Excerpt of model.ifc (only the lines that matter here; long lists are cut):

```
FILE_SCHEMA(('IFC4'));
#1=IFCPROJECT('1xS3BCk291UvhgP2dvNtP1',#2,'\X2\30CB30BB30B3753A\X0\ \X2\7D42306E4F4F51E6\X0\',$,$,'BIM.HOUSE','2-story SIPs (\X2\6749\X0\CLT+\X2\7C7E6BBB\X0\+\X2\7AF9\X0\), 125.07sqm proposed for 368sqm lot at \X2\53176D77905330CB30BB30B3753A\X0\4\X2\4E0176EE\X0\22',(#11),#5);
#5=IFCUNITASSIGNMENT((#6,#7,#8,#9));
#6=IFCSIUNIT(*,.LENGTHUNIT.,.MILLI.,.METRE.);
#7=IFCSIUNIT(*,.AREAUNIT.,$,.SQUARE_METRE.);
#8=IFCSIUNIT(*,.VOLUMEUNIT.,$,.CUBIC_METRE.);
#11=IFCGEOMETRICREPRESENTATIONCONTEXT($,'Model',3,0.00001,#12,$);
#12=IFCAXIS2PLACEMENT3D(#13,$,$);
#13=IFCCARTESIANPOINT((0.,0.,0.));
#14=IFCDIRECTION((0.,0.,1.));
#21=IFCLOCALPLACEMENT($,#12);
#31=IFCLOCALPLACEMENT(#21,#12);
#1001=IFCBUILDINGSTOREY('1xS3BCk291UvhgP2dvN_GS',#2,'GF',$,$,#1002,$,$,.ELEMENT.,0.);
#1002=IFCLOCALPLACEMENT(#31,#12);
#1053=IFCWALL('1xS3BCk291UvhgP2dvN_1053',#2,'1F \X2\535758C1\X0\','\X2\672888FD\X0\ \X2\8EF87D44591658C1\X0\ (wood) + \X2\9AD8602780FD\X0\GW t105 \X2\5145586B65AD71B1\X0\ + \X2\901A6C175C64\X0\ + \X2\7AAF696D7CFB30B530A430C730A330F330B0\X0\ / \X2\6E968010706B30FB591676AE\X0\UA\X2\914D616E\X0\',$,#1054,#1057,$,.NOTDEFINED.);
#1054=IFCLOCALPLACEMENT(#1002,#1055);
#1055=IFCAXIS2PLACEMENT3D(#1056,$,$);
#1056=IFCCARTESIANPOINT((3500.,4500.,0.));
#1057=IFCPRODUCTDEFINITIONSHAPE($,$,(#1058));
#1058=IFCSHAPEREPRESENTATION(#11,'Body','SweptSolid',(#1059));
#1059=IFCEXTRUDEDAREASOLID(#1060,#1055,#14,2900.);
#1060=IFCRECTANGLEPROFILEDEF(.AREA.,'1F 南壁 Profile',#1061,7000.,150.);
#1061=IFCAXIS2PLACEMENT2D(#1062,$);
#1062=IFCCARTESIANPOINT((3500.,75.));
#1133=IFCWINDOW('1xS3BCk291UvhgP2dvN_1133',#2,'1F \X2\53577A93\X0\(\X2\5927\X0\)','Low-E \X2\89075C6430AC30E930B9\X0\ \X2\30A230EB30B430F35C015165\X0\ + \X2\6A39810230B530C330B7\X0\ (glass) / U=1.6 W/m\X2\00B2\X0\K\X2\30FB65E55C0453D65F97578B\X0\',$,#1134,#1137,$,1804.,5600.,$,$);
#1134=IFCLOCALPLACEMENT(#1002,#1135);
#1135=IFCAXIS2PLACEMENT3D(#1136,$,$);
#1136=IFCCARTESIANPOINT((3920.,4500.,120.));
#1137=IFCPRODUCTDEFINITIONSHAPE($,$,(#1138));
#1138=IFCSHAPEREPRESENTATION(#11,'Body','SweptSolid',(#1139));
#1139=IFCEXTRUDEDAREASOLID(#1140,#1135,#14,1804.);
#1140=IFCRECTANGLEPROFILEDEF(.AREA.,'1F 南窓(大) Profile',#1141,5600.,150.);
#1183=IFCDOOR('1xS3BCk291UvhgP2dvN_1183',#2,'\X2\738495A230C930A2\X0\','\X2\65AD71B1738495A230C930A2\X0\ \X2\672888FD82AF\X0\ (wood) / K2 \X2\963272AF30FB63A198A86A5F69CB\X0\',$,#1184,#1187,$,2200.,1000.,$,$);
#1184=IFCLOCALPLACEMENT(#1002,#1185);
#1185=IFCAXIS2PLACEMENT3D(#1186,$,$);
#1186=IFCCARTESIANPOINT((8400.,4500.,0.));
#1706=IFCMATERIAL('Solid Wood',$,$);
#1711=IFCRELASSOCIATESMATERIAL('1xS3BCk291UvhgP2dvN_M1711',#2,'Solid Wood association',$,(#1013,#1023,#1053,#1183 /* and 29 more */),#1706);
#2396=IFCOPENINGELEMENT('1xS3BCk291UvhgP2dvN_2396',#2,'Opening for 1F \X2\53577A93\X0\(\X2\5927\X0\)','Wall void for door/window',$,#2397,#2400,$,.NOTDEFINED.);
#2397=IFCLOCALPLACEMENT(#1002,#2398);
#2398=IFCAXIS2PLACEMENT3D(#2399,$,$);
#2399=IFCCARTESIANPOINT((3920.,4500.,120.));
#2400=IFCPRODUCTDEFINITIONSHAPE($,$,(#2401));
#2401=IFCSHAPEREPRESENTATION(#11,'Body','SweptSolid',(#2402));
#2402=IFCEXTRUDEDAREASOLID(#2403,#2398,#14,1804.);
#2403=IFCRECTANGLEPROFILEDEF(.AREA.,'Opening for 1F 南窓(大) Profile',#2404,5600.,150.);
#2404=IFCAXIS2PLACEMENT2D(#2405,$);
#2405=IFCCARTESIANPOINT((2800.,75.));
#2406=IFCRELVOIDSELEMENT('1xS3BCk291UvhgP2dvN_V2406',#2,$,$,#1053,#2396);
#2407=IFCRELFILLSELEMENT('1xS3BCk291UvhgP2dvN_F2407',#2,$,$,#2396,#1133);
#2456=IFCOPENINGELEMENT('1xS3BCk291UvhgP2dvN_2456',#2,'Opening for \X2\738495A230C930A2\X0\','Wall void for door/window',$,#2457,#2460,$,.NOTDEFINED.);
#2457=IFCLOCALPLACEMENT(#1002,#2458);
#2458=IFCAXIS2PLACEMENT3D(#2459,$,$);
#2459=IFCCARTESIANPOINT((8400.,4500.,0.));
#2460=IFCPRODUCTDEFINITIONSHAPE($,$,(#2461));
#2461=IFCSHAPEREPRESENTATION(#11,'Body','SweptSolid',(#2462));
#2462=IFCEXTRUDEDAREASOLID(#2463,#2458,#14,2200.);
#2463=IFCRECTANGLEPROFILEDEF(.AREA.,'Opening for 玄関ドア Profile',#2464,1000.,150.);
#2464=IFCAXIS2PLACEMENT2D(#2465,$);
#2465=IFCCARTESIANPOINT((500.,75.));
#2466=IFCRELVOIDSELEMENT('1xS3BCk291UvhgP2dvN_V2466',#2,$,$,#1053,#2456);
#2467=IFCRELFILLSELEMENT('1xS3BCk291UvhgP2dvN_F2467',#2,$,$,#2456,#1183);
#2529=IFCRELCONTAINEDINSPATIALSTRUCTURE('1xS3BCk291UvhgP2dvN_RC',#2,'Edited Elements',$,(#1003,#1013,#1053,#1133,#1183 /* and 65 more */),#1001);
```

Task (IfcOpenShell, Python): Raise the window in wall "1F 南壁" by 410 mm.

```python
import numpy as np
import ifcopenshell
import ifcopenshell.api.geometry
import ifcopenshell.util.placement
import ifcopenshell.util.unit

model = ifcopenshell.open("model.ifc")
unit_scale = ifcopenshell.util.unit.calculate_unit_scale(model)

window = model.by_id(1133)
opening = window.FillsVoids[0].RelatingOpeningElement
dz = 0.41 / unit_scale

shift = np.array([0.0, 0.0, dz])
# The window is not placed relative to its opening, so move both.
for product in (opening, window):
    matrix = ifcopenshell.util.placement.get_local_placement(product.ObjectPlacement)
    matrix[:3, 3] += shift
    ifcopenshell.api.geometry.edit_object_placement(model, product=product, matrix=matrix, is_si=False)

print(f"moved by {dz * unit_scale:+.3f} m")

model.write("model_v2.ifc")
```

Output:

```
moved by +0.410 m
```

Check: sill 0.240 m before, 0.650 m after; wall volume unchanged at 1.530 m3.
